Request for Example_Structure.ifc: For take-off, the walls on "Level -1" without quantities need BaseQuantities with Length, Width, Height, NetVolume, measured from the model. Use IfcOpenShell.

First a look at what the model holds.

```python
import ifcopenshell
import ifcopenshell.util.element
import ifcopenshell.util.unit

model = ifcopenshell.open("Example_Structure.ifc")
print(model.schema)
for unit_type in ("LENGTHUNIT", "AREAUNIT", "VOLUMEUNIT"):
    print(unit_type, ifcopenshell.util.unit.calculate_unit_scale(model, unit_type))
storey = next(s for s in model.by_type("IfcBuildingStorey") if s.Name == "Level -1")
walls = [e for e in ifcopenshell.util.element.get_decomposition(storey) if e.is_a("IfcWall")]
for e in sorted(walls, key=lambda e: e.id()):
    print(e.id(), e.is_a(), e.Name, list(ifcopenshell.util.element.get_psets(e, qtos_only=True)), sep=" | ")
```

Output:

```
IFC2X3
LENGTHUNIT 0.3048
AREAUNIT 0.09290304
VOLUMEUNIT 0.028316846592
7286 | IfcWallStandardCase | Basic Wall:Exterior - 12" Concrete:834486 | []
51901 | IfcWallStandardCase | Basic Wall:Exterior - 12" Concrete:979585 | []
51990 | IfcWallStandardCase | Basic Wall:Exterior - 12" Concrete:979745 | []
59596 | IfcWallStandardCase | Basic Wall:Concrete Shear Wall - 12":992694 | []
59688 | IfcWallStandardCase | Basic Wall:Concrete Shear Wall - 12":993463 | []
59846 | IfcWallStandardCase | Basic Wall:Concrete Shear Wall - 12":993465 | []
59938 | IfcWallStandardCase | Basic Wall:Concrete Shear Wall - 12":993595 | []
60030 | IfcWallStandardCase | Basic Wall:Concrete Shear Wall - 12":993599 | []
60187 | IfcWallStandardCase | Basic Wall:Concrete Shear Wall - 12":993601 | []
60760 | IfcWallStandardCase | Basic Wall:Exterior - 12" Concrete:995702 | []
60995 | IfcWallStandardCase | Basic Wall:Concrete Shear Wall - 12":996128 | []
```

```python
import ifcopenshell
import ifcopenshell.api.pset
import ifcopenshell.geom
import ifcopenshell.util.element
import ifcopenshell.util.shape
import ifcopenshell.util.unit

model = ifcopenshell.open("Example_Structure.ifc")
unit_scale = ifcopenshell.util.unit.calculate_unit_scale(model)
volume_scale = ifcopenshell.util.unit.calculate_unit_scale(model, "VOLUMEUNIT")
settings = ifcopenshell.geom.settings()

storey = next(s for s in model.by_type("IfcBuildingStorey") if s.Name == "Level -1")
walls = [e for e in ifcopenshell.util.element.get_decomposition(storey) if e.is_a("IfcWall")]

for e in sorted(walls, key=lambda e: e.id()):
    if ifcopenshell.util.element.get_psets(e, qtos_only=True, should_inherit=False):
        continue
    # Geometry comes back in metres, in the element's own axes.
    shape = ifcopenshell.geom.create_shape(settings, e)
    values = {
        "Length": ifcopenshell.util.shape.get_x(shape.geometry) / unit_scale,
        "Width": ifcopenshell.util.shape.get_y(shape.geometry) / unit_scale,
        "Height": ifcopenshell.util.shape.get_z(shape.geometry) / unit_scale,
        "NetVolume": ifcopenshell.util.shape.get_volume(shape.geometry) / volume_scale,
    }
    qto = ifcopenshell.api.pset.add_qto(model, product=e, name="BaseQuantities")
    ifcopenshell.api.pset.edit_qto(model, qto=qto, properties=values)
    print(e.id(), {k: round(v, 3) for k, v in values.items()})

model.write("Example_Structure_updated.ifc")
```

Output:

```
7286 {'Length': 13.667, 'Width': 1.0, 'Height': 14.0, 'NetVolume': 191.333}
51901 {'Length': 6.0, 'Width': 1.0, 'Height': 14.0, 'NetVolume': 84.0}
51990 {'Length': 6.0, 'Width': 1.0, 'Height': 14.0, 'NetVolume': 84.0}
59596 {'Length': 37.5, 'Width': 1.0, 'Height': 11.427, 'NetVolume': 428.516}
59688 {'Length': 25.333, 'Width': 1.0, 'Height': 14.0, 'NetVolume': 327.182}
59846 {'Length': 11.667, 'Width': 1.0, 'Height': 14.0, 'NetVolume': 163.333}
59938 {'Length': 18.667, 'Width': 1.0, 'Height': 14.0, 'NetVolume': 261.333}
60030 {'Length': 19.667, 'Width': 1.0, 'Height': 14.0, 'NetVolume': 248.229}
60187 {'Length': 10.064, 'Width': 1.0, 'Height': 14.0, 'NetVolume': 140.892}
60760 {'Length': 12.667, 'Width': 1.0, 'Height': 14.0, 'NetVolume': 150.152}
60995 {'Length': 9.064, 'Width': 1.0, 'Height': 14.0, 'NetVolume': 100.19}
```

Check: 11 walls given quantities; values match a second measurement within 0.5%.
